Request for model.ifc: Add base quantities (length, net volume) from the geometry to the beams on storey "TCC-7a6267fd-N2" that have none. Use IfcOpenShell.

First a look at what the model holds.

```python
import ifcopenshell
import ifcopenshell.util.element
import ifcopenshell.util.unit

model = ifcopenshell.open("model.ifc")
print(model.schema)
for unit_type in ("LENGTHUNIT", "AREAUNIT", "VOLUMEUNIT"):
    print(unit_type, ifcopenshell.util.unit.calculate_unit_scale(model, unit_type))
storey = next(s for s in model.by_type("IfcBuildingStorey") if s.Name == "TCC-7a6267fd-N2")
beams = [e for e in ifcopenshell.util.element.get_decomposition(storey) if e.is_a("IfcBeam")]
for e in sorted(beams, key=lambda e: e.id()):
    print(e.id(), e.is_a(), e.Name, list(ifcopenshell.util.element.get_psets(e, qtos_only=True)), sep=" | ")
```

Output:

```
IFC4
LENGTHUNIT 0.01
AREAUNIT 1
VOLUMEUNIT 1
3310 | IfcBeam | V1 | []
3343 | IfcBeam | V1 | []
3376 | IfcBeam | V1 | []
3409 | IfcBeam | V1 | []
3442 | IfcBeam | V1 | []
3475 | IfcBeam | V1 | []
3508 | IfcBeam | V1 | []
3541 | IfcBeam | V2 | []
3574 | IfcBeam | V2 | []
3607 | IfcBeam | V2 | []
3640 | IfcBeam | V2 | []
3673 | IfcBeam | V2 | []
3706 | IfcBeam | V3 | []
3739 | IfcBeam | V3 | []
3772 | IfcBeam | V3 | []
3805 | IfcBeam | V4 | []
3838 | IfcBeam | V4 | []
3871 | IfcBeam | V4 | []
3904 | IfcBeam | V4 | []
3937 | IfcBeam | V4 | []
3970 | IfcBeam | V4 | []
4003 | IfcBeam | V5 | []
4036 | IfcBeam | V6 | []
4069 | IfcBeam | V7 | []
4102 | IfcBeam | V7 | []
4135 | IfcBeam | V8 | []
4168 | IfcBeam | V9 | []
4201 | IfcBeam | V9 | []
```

```python
import ifcopenshell
import ifcopenshell.api.pset
import ifcopenshell.geom
import ifcopenshell.util.element
import ifcopenshell.util.shape
import ifcopenshell.util.unit

model = ifcopenshell.open("model.ifc")
unit_scale = ifcopenshell.util.unit.calculate_unit_scale(model)
volume_scale = ifcopenshell.util.unit.calculate_unit_scale(model, "VOLUMEUNIT")
settings = ifcopenshell.geom.settings()

storey = next(s for s in model.by_type("IfcBuildingStorey") if s.Name == "TCC-7a6267fd-N2")
beams = [e for e in ifcopenshell.util.element.get_decomposition(storey) if e.is_a("IfcBeam")]

for e in sorted(beams, key=lambda e: e.id()):
    if ifcopenshell.util.element.get_psets(e, qtos_only=True, should_inherit=False):
        continue
    # Geometry comes back in metres, in the element's own axes.
    shape = ifcopenshell.geom.create_shape(settings, e)
    values = {
        "Length": ifcopenshell.util.shape.get_max_xyz(shape.geometry) / unit_scale,
        "NetVolume": ifcopenshell.util.shape.get_volume(shape.geometry) / volume_scale,
    }
    qto = ifcopenshell.api.pset.add_qto(model, product=e, name="Qto_BeamBaseQuantities")
    ifcopenshell.api.pset.edit_qto(model, qto=qto, properties=values)
    print(e.id(), {k: round(v, 3) for k, v in values.items()})

model.write("model_rev.ifc")
```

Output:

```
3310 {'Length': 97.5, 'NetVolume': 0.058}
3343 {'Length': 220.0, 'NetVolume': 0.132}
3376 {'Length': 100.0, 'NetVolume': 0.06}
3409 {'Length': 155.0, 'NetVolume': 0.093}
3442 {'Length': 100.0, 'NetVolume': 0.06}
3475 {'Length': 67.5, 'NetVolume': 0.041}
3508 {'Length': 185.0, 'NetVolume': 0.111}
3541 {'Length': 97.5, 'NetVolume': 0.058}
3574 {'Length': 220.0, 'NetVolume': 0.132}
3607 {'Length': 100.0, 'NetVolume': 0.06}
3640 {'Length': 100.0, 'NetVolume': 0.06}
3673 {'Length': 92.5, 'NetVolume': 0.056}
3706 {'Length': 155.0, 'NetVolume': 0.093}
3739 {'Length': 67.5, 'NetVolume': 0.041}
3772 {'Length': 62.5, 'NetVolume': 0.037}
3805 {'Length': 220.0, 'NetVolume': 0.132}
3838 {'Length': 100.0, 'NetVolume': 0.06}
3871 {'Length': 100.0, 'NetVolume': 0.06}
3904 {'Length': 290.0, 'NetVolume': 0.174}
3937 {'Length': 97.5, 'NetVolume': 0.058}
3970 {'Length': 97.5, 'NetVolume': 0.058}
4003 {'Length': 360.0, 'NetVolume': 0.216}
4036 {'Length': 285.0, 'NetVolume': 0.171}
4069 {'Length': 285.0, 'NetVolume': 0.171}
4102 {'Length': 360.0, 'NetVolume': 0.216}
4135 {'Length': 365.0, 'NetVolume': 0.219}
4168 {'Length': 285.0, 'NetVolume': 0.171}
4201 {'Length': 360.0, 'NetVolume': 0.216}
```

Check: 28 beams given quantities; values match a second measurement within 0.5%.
